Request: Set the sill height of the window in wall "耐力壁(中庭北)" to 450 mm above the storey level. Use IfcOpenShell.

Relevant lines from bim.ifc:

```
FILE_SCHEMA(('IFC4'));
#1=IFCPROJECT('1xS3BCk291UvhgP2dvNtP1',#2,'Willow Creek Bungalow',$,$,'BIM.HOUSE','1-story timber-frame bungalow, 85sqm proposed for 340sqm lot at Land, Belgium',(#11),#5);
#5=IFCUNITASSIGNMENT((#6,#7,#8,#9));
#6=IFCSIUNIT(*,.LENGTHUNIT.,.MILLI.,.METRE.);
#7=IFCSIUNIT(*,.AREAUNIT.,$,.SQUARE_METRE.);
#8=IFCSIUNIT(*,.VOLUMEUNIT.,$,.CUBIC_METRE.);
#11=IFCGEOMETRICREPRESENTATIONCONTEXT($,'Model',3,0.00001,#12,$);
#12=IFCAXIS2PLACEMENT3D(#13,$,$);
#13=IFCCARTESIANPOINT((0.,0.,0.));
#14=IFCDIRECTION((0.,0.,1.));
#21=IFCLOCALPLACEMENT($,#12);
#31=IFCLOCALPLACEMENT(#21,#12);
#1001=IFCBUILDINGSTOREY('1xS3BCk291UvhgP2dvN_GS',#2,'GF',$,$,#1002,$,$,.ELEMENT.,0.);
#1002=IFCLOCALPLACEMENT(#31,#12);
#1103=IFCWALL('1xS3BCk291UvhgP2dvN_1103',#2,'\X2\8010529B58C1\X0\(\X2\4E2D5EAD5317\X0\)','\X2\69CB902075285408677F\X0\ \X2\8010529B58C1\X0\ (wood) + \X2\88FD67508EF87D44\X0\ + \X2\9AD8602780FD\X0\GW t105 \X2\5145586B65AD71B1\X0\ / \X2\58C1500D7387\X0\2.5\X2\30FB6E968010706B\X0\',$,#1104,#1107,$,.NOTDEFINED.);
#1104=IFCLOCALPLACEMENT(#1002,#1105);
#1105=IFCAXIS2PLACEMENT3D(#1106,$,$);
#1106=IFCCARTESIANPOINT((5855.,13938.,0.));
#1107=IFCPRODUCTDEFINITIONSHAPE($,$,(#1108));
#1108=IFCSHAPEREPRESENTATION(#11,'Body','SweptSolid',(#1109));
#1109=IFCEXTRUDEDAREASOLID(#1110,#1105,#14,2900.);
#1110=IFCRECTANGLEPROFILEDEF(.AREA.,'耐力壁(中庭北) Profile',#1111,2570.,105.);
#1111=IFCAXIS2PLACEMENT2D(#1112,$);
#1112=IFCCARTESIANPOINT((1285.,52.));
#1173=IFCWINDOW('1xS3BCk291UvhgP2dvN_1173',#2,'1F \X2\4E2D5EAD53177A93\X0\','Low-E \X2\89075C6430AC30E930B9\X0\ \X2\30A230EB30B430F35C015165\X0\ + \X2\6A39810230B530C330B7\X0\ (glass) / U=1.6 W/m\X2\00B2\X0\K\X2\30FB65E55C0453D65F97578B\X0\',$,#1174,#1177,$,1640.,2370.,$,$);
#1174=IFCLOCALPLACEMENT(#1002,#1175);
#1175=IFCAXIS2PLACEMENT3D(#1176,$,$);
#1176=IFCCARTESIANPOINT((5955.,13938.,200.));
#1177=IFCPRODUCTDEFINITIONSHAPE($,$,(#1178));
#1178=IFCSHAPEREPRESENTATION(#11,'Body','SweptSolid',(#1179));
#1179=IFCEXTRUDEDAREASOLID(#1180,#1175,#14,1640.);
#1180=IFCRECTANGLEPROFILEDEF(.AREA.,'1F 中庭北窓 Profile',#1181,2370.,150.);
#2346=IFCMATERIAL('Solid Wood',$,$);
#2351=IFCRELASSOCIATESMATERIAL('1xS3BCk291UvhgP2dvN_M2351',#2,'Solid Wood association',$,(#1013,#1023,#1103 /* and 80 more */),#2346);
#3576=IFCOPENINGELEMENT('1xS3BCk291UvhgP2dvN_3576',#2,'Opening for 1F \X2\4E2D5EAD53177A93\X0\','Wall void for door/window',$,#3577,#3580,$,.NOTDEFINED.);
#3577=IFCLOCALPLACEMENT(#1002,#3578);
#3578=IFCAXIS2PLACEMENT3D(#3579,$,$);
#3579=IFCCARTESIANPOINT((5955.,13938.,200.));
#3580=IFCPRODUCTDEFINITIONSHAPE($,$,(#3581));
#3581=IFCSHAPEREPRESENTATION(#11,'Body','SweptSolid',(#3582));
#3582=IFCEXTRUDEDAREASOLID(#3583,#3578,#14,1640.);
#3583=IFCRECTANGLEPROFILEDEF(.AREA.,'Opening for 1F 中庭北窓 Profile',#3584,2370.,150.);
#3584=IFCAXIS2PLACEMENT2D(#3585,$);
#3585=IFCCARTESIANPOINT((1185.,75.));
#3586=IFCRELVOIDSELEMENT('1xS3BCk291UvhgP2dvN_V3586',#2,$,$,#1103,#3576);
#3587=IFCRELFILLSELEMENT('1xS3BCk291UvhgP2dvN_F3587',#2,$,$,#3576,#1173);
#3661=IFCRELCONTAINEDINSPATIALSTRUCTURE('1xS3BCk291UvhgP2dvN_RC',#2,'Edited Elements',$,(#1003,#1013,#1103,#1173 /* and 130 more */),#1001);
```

```python
import numpy as np
import ifcopenshell
import ifcopenshell.api.geometry
import ifcopenshell.geom
import ifcopenshell.util.element
import ifcopenshell.util.placement
import ifcopenshell.util.shape
import ifcopenshell.util.unit

model = ifcopenshell.open("bim.ifc")
unit_scale = ifcopenshell.util.unit.calculate_unit_scale(model)

window = model.by_id(1173)
opening = window.FillsVoids[0].RelatingOpeningElement
storey = ifcopenshell.util.element.get_container(window, ifc_class="IfcBuildingStorey")
level = ifcopenshell.util.placement.get_local_placement(storey.ObjectPlacement)[2, 3]

# The opening's origin need not be at the sill, so measure its lowest point.
shape = ifcopenshell.geom.create_shape(ifcopenshell.geom.settings(), opening)
bottom = ifcopenshell.util.shape.get_shape_bottom_elevation(shape, shape.geometry) / unit_scale
dz = level + 450.0 - bottom

shift = np.array([0.0, 0.0, dz])
# The window is not placed relative to its opening, so move both.
for product in (opening, window):
    matrix = ifcopenshell.util.placement.get_local_placement(product.ObjectPlacement)
    matrix[:3, 3] += shift
    ifcopenshell.api.geometry.edit_object_placement(model, product=product, matrix=matrix, is_si=False)

print(f"moved by {dz * unit_scale:+.3f} m")

model.write("bim_v2.ifc")
```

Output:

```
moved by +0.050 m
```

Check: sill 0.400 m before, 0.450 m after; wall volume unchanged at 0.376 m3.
